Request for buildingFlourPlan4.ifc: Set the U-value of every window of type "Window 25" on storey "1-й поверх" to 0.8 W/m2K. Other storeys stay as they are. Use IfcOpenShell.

First a look at what the model holds.

```python
import ifcopenshell
import ifcopenshell.util.element

model = ifcopenshell.open("buildingFlourPlan4.ifc")
print(model.schema)
storey = next(s for s in model.by_type("IfcBuildingStorey") if s.Name == "1-й поверх")
windows = [e for e in ifcopenshell.util.element.get_decomposition(storey) if e.is_a("IfcWindow")]
seen = {}
for e in windows:
    element_type = ifcopenshell.util.element.get_type(e)
    key = (element_type.Name if element_type != e and element_type else None, ifcopenshell.util.element.get_pset(e, "Pset_WindowCommon", "ThermalTransmittance"))
    seen[key] = seen.get(key, 0) + 1
for (name, value), count in sorted(seen.items(), key=str):
    print(count, "x", name, "|", value)
```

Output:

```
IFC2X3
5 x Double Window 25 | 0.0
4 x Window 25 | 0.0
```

```python
import ifcopenshell
import ifcopenshell.api.pset
import ifcopenshell.util.element

model = ifcopenshell.open("buildingFlourPlan4.ifc")

storey = next(s for s in model.by_type("IfcBuildingStorey") if s.Name == "1-й поверх")
windows = [e for e in ifcopenshell.util.element.get_decomposition(storey) if e.is_a("IfcWindow")]

count = 0
for e in windows:
    element_type = ifcopenshell.util.element.get_type(e)
    if element_type in (None, e) or element_type.Name != "Window 25":
        continue
    # add_pset returns the element's existing set when there is one.
    pset = ifcopenshell.api.pset.add_pset(model, product=e, name="Pset_WindowCommon")
    ifcopenshell.api.pset.edit_pset(model, pset=pset, properties={"ThermalTransmittance": 0.8})
    count += 1

print(count, "windows updated")

model.write("buildingFlourPlan4-out.ifc")
```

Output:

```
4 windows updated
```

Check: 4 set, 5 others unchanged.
